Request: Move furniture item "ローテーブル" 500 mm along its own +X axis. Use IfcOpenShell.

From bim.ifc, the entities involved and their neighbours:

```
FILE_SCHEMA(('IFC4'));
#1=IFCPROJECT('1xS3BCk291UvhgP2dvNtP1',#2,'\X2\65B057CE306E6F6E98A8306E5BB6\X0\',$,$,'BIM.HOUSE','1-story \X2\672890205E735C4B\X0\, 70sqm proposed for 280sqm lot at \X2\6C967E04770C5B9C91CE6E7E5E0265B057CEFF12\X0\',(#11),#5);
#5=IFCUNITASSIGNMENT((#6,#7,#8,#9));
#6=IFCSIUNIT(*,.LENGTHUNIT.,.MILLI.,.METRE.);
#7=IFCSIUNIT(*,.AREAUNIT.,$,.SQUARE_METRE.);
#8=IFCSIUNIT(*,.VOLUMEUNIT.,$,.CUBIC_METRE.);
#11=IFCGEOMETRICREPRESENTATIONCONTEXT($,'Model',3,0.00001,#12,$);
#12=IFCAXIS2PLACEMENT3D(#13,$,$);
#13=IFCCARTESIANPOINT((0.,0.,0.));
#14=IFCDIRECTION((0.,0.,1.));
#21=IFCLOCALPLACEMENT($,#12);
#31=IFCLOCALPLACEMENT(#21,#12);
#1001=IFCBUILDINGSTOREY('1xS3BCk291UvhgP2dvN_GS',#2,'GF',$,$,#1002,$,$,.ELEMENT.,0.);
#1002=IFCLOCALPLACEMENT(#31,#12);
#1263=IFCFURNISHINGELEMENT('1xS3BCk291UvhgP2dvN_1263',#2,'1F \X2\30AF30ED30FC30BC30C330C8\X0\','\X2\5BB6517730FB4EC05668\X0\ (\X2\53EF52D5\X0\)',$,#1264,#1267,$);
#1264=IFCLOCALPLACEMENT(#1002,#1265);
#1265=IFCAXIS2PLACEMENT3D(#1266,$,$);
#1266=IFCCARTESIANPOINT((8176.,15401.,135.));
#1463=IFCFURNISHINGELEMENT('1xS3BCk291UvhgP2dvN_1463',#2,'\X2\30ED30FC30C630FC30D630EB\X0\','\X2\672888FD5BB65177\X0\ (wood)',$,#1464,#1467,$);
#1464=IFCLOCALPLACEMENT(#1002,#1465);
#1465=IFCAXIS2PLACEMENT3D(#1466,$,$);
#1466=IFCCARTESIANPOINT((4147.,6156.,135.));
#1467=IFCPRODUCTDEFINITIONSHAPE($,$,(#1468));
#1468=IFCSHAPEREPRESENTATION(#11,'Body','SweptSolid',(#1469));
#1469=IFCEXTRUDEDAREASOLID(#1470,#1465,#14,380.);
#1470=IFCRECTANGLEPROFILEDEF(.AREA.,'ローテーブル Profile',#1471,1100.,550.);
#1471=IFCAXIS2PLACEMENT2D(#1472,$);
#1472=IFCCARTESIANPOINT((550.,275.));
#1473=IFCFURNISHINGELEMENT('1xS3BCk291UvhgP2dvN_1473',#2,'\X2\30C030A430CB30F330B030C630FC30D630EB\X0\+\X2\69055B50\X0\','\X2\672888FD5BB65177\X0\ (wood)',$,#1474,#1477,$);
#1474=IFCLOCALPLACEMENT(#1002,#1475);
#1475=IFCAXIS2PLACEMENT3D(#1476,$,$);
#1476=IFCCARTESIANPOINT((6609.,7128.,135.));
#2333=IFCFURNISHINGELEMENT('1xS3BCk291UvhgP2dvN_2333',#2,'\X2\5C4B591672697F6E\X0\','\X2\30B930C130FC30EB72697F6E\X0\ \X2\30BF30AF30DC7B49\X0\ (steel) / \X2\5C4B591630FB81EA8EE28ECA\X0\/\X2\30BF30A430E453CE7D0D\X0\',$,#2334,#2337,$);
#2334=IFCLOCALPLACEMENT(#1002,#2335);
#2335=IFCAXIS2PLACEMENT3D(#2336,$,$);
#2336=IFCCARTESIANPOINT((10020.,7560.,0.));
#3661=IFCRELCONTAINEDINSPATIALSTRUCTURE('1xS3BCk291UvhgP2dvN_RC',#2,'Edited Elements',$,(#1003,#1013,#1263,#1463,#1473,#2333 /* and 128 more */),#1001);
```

```python
import ifcopenshell
import ifcopenshell.api.geometry
import ifcopenshell.util.placement

model = ifcopenshell.open("bim.ifc")

item = model.by_id(1463)
matrix = ifcopenshell.util.placement.get_local_placement(item.ObjectPlacement)
matrix[:3, 3] += matrix[:3, 0] * 500.0
ifcopenshell.api.geometry.edit_object_placement(model, product=item, matrix=matrix, is_si=False)

print(ifcopenshell.util.placement.get_local_placement(item.ObjectPlacement).round(3) + 0.0)

model.write("bim-out.ifc")
```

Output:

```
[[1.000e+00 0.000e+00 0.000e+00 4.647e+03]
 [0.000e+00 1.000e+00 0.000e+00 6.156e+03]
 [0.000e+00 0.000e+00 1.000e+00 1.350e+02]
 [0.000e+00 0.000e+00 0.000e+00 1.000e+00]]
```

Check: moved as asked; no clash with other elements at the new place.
